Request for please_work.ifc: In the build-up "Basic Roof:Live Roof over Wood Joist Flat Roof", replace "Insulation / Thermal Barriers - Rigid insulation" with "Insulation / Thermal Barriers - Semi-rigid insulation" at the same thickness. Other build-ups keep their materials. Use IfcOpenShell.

First a look at what the model holds.

```python
import ifcopenshell
import ifcopenshell.util.element

model = ifcopenshell.open("please_work.ifc")
print(model.schema)
for layer_set in model.by_type("IfcMaterialLayerSet"):
    if layer_set.LayerSetName == "Basic Roof:Live Roof over Wood Joist Flat Roof":
        for layer in layer_set.MaterialLayers:
            print(layer.id(), layer.Material and layer.Material.Name, layer.LayerThickness, sep=" | ")
        print(len(ifcopenshell.util.element.get_elements_by_material(model, layer_set)), "elements and types use it")
print(sorted(m.Name for m in model.by_type("IfcMaterial") if m.Name)[:60])
```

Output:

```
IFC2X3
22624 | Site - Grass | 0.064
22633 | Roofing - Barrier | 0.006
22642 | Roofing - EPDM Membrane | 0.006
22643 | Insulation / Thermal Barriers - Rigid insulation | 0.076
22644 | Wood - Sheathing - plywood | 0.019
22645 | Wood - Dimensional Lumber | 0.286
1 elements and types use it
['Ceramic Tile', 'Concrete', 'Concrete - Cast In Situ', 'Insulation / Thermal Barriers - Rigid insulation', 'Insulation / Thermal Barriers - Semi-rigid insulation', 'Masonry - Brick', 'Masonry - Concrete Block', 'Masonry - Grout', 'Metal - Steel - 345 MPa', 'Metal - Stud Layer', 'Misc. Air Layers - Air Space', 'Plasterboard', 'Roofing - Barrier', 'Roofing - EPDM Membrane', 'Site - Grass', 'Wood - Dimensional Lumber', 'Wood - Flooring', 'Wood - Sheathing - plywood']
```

```python
import ifcopenshell
import ifcopenshell.api.material

model = ifcopenshell.open("please_work.ifc")

layer_set = next(s for s in model.by_type("IfcMaterialLayerSet") if s.LayerSetName == "Basic Roof:Live Roof over Wood Joist Flat Roof")
layer = next(l for l in layer_set.MaterialLayers if l.Material and l.Material.Name == "Insulation / Thermal Barriers - Rigid insulation")
material = next(m for m in model.by_type("IfcMaterial") if m.Name == "Insulation / Thermal Barriers - Semi-rigid insulation")

# Point this one layer at the other material; renaming the old one would change it everywhere.
ifcopenshell.api.material.edit_layer(model, layer=layer, attributes={}, material=material)

print([l.Material.Name if l.Material else None for l in layer_set.MaterialLayers])

model.write("please_work_edited.ifc")
```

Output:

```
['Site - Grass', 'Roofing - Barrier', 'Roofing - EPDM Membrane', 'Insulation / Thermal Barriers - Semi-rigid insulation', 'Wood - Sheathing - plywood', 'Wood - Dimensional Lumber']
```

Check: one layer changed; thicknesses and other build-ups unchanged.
